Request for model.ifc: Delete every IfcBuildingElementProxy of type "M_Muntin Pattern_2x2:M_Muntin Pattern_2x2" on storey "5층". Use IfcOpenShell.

First a look at what the model holds.

```python
import ifcopenshell
import ifcopenshell.util.element

model = ifcopenshell.open("model.ifc")
print(model.schema)
storey = next(s for s in model.by_type("IfcBuildingStorey") if s.Name == "5층")
proxies = [e for e in ifcopenshell.util.element.get_decomposition(storey) if e.is_a("IfcBuildingElementProxy")]
seen = {}
for e in proxies:
    element_type = ifcopenshell.util.element.get_type(e)
    name = element_type.Name if element_type not in (None, e) else None
    seen[name] = seen.get(name, 0) + 1
for name, count in sorted(seen.items(), key=str):
    print(count, "x", name)
```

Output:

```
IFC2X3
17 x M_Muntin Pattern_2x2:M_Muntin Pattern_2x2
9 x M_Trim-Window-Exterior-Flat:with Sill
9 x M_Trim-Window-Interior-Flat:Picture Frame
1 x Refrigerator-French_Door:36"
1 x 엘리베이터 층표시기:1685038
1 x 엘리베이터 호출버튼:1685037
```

```python
import ifcopenshell
import ifcopenshell.api.root
import ifcopenshell.util.element

model = ifcopenshell.open("model.ifc")

storey = next(s for s in model.by_type("IfcBuildingStorey") if s.Name == "5층")
proxies = [e for e in ifcopenshell.util.element.get_decomposition(storey) if e.is_a("IfcBuildingElementProxy")]
targets = [e for e in proxies if (t := ifcopenshell.util.element.get_type(e)) not in (None, e) and t.Name == "M_Muntin Pattern_2x2:M_Muntin Pattern_2x2"]

for e in targets:
    ifcopenshell.api.root.remove_product(model, product=e)
print(len(targets), "removed")

model.write("model_rev.ifc")
```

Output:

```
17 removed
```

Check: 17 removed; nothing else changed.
